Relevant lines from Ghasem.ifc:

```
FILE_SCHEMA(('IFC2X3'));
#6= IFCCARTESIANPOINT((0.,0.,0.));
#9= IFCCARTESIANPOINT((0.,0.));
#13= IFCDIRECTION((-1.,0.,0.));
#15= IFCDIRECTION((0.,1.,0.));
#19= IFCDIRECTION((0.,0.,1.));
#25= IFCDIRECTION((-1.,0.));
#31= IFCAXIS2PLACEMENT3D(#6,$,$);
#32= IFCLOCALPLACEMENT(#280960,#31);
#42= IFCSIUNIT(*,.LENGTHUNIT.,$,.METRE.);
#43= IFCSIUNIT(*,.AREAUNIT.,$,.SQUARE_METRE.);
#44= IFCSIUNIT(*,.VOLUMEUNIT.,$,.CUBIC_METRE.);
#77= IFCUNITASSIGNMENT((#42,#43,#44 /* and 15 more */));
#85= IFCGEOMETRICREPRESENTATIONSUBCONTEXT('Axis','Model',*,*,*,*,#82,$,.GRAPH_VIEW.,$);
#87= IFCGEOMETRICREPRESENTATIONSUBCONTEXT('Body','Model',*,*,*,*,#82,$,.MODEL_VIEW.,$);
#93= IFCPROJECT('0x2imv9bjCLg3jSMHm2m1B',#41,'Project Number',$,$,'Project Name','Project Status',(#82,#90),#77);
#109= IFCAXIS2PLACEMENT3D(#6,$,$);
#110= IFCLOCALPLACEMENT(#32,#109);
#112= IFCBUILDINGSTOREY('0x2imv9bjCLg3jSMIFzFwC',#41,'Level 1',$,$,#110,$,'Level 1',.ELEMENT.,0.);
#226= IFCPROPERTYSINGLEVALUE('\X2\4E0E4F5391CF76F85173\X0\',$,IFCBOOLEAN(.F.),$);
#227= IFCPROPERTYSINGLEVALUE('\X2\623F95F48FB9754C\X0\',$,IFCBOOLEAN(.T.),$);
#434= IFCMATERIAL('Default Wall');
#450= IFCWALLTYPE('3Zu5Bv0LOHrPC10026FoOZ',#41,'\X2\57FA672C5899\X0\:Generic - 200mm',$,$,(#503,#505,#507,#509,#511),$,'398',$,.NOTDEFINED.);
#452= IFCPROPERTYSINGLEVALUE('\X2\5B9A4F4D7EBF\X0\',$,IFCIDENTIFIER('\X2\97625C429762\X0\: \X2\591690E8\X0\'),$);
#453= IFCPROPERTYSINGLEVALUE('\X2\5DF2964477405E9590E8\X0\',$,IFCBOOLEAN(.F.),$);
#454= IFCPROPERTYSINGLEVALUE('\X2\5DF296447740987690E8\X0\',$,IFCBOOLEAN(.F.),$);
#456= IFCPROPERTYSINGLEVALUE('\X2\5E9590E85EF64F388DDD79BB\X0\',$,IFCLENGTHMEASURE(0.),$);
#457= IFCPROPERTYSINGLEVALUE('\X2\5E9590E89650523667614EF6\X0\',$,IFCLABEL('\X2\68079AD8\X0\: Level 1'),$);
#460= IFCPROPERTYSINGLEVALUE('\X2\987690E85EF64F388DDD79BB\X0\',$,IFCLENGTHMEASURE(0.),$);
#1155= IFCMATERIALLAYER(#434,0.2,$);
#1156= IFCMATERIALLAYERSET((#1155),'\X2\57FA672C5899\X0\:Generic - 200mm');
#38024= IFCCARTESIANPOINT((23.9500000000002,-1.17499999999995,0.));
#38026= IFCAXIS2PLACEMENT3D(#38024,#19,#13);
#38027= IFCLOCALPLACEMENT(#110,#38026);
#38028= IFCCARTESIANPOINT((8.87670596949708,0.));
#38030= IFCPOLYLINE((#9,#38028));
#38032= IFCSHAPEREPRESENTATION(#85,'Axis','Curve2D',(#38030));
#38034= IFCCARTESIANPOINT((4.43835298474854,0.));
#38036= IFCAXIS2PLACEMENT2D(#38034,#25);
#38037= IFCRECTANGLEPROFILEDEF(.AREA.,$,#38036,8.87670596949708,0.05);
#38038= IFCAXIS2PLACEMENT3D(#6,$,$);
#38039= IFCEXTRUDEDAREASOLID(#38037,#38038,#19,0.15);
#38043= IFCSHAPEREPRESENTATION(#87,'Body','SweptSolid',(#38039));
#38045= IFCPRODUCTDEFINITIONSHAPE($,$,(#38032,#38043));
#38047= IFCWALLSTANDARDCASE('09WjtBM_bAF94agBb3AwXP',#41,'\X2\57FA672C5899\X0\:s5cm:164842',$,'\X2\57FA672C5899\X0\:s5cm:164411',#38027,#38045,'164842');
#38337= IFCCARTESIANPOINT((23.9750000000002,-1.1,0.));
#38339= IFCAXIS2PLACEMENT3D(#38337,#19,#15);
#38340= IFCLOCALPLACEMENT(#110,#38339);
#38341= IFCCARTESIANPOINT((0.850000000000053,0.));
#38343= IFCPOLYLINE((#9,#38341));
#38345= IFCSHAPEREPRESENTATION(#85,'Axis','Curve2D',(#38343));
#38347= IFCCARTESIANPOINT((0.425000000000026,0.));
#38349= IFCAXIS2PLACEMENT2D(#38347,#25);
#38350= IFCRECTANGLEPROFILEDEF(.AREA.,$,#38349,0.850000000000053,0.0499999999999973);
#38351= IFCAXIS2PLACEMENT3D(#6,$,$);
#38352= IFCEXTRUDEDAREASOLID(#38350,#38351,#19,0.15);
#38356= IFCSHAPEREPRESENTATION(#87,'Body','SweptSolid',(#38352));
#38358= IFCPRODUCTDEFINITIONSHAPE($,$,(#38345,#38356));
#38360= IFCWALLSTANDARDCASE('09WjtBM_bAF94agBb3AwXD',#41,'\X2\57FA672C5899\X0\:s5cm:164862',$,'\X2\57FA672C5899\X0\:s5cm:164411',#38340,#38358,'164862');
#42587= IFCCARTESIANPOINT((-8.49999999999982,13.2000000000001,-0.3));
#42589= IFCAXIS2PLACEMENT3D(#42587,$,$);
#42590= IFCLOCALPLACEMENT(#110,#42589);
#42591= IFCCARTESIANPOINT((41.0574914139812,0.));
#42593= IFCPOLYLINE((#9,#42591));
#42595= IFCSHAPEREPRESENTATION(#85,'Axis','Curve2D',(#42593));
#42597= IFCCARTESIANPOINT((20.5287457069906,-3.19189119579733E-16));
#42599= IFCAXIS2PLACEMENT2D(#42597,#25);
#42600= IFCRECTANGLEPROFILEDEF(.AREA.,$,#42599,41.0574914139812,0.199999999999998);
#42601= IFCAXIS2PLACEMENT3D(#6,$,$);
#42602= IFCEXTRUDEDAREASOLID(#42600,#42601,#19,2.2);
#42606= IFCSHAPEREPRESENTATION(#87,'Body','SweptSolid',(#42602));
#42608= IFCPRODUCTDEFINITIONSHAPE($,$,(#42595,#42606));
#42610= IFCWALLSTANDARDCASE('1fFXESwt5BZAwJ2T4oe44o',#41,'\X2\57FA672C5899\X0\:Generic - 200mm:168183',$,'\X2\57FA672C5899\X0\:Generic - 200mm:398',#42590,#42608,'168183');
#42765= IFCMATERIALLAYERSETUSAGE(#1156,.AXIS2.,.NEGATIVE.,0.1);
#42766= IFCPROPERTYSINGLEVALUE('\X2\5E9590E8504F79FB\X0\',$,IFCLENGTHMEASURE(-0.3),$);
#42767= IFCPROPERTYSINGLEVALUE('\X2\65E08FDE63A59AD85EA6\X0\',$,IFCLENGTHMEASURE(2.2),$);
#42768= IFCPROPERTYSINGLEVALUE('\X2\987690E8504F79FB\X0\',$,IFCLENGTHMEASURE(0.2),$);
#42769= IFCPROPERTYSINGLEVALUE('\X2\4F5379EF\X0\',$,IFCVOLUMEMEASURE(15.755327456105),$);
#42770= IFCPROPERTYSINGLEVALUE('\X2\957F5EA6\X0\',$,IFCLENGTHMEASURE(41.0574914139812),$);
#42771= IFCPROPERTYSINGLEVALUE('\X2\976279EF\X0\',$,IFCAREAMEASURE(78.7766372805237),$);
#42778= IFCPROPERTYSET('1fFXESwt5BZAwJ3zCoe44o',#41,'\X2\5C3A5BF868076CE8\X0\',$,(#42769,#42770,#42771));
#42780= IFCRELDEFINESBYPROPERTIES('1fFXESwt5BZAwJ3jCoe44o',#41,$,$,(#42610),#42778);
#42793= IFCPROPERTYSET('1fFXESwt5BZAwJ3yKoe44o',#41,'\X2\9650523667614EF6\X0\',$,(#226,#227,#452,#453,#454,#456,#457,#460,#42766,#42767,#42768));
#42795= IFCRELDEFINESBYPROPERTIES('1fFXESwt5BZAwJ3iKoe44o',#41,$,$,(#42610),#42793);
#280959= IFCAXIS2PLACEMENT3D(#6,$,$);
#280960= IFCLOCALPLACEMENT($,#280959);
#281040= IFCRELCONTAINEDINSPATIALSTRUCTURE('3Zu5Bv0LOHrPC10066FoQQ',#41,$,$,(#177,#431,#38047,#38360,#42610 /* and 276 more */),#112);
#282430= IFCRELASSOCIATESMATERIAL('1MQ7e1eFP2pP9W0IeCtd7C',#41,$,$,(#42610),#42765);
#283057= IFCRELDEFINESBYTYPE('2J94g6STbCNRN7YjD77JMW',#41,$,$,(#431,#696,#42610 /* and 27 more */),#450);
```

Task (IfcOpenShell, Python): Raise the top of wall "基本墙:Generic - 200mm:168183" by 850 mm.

```python
import ifcopenshell
import ifcopenshell.api.pset
import ifcopenshell.geom
import ifcopenshell.util.element
import ifcopenshell.util.representation
import ifcopenshell.util.shape
import ifcopenshell.util.unit

model = ifcopenshell.open("Ghasem.ifc")
area_scale = ifcopenshell.util.unit.calculate_unit_scale(model, "AREAUNIT")
volume_scale = ifcopenshell.util.unit.calculate_unit_scale(model, "VOLUMEUNIT")
settings = ifcopenshell.geom.settings()


def volume(element):
    """Net volume in cubic metres, openings subtracted."""
    shape = ifcopenshell.geom.create_shape(settings, element)
    return ifcopenshell.util.shape.get_volume(shape.geometry)


wall = model.by_guid("1fFXESwt5BZAwJ2T4oe44o")
before = volume(wall)

body = ifcopenshell.util.representation.get_representation(wall, "Model", "Body")
solid = body.Items[0]
old_height = solid.Depth
solid.Depth += 0.85
after = volume(wall)
thickness = 0.2  # wall thickness in metres

# Update the stored height, areas and volumes.
pset = model.by_id(ifcopenshell.util.element.get_pset(wall, "尺寸标注", should_inherit=False)["id"])
ifcopenshell.api.pset.edit_pset(model, pset=pset, properties={
    "体积": model.create_entity("IfcVolumeMeasure", after / volume_scale),
    "面积": model.create_entity("IfcAreaMeasure", after / thickness / area_scale),
})
pset = model.by_id(ifcopenshell.util.element.get_pset(wall, "限制条件", should_inherit=False)["id"])
ifcopenshell.api.pset.edit_pset(model, pset=pset, properties={
    "无连接高度": model.create_entity("IfcLengthMeasure", solid.Depth),
})

print(f"height {old_height:g} -> {solid.Depth:g}, volume {before:.3f} -> {after:.3f} m3")

model.write("Ghasem_updated.ifc")
```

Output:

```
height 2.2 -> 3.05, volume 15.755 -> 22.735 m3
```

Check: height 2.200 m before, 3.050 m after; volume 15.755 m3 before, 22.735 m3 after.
